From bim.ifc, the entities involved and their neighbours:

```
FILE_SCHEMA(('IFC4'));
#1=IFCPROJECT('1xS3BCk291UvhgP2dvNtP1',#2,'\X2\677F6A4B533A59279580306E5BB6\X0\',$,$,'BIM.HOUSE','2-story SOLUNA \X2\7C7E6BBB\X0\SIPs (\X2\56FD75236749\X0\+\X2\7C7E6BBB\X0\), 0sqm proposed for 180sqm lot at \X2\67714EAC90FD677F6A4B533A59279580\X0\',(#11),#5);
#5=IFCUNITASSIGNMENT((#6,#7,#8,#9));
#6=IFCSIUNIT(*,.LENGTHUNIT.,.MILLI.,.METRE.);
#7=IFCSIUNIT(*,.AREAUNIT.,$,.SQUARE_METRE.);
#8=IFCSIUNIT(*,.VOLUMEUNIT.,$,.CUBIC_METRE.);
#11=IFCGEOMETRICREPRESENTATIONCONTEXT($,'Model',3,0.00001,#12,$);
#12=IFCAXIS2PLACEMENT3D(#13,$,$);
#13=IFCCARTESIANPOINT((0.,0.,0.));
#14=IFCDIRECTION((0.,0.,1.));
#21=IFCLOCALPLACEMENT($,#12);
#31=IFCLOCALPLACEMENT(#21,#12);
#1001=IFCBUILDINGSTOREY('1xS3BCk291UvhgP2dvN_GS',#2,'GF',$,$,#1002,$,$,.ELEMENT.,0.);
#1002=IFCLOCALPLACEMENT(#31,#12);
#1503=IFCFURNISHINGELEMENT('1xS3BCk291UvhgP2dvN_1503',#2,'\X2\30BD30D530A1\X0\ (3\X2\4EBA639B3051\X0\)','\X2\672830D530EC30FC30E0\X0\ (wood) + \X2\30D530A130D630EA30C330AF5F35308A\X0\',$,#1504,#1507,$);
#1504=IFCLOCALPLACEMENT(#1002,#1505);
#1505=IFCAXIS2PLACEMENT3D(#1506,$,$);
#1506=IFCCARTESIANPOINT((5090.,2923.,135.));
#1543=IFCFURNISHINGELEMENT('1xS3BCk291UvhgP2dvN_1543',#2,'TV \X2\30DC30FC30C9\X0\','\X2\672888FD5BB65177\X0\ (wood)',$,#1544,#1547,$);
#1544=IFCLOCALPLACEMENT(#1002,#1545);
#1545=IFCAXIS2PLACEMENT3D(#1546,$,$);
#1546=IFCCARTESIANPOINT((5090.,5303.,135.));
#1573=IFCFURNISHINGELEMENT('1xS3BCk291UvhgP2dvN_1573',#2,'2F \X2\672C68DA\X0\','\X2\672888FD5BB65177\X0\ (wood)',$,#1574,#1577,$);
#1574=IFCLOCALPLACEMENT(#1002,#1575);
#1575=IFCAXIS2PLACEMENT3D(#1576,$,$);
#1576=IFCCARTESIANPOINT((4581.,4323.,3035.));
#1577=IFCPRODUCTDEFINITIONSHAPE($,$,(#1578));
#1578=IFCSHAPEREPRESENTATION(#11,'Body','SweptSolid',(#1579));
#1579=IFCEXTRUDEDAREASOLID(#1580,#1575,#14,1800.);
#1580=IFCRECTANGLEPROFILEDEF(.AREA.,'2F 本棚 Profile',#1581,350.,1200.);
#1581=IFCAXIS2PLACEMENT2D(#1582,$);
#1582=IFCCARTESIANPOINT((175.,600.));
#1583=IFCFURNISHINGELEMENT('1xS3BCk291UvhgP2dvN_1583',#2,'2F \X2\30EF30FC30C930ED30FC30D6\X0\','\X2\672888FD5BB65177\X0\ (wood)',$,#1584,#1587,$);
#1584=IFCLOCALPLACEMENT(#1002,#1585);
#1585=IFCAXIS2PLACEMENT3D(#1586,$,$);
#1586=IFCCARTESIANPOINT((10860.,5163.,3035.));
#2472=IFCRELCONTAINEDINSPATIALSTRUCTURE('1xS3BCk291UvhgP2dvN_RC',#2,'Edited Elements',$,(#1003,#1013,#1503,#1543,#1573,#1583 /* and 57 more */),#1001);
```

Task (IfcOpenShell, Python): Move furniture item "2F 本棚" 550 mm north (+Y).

```python
import ifcopenshell
import ifcopenshell.api.geometry
import ifcopenshell.util.placement

model = ifcopenshell.open("bim.ifc")

item = model.by_guid("1xS3BCk291UvhgP2dvN_1573")
matrix = ifcopenshell.util.placement.get_local_placement(item.ObjectPlacement)
matrix[1, 3] += 550.0
ifcopenshell.api.geometry.edit_object_placement(model, product=item, matrix=matrix, is_si=False)

print(ifcopenshell.util.placement.get_local_placement(item.ObjectPlacement).round(3) + 0.0)

model.write("bim_v2.ifc")
```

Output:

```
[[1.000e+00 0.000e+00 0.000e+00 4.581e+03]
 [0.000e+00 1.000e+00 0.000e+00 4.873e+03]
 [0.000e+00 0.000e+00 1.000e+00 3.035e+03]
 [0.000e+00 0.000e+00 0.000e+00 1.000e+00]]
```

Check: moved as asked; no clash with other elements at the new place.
